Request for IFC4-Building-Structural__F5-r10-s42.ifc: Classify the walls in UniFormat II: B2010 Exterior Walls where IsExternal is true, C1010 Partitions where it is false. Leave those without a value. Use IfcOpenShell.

First a look at what the model holds.

```python
import ifcopenshell
import ifcopenshell.util.element

model = ifcopenshell.open("IFC4-Building-Structural__F5-r10-s42.ifc")
print(model.schema)
print("classifications:", [c.Name for c in model.by_type("IfcClassification")])
values = [ifcopenshell.util.element.get_pset(e, "Pset_WallCommon", "IsExternal") for e in model.by_type("IfcWall")]
for value in (True, False, None):
    print("IsExternal", value, values.count(value))
```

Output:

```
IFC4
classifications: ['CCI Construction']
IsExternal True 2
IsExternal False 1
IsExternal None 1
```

```python
import ifcopenshell
import ifcopenshell.api.classification
import ifcopenshell.util.element

model = ifcopenshell.open("IFC4-Building-Structural__F5-r10-s42.ifc")

system = ifcopenshell.api.classification.add_classification(model, classification="UniFormat II")

walls = model.by_type("IfcWall")
external = {e: ifcopenshell.util.element.get_pset(e, "Pset_WallCommon", "IsExternal") for e in walls}
for flag, code, name in ((True, "B2010", "Exterior Walls"), (False, "C1010", "Partitions")):
    products = [e for e in walls if external[e] is flag]
    ifcopenshell.api.classification.add_reference(
        model, products=products, classification=system, identification=code, name=name
    )
    print(code, len(products))

model.write("IFC4-Building-Structural__F5-r10-s42-out.ifc")
```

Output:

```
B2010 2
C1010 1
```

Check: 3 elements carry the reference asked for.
